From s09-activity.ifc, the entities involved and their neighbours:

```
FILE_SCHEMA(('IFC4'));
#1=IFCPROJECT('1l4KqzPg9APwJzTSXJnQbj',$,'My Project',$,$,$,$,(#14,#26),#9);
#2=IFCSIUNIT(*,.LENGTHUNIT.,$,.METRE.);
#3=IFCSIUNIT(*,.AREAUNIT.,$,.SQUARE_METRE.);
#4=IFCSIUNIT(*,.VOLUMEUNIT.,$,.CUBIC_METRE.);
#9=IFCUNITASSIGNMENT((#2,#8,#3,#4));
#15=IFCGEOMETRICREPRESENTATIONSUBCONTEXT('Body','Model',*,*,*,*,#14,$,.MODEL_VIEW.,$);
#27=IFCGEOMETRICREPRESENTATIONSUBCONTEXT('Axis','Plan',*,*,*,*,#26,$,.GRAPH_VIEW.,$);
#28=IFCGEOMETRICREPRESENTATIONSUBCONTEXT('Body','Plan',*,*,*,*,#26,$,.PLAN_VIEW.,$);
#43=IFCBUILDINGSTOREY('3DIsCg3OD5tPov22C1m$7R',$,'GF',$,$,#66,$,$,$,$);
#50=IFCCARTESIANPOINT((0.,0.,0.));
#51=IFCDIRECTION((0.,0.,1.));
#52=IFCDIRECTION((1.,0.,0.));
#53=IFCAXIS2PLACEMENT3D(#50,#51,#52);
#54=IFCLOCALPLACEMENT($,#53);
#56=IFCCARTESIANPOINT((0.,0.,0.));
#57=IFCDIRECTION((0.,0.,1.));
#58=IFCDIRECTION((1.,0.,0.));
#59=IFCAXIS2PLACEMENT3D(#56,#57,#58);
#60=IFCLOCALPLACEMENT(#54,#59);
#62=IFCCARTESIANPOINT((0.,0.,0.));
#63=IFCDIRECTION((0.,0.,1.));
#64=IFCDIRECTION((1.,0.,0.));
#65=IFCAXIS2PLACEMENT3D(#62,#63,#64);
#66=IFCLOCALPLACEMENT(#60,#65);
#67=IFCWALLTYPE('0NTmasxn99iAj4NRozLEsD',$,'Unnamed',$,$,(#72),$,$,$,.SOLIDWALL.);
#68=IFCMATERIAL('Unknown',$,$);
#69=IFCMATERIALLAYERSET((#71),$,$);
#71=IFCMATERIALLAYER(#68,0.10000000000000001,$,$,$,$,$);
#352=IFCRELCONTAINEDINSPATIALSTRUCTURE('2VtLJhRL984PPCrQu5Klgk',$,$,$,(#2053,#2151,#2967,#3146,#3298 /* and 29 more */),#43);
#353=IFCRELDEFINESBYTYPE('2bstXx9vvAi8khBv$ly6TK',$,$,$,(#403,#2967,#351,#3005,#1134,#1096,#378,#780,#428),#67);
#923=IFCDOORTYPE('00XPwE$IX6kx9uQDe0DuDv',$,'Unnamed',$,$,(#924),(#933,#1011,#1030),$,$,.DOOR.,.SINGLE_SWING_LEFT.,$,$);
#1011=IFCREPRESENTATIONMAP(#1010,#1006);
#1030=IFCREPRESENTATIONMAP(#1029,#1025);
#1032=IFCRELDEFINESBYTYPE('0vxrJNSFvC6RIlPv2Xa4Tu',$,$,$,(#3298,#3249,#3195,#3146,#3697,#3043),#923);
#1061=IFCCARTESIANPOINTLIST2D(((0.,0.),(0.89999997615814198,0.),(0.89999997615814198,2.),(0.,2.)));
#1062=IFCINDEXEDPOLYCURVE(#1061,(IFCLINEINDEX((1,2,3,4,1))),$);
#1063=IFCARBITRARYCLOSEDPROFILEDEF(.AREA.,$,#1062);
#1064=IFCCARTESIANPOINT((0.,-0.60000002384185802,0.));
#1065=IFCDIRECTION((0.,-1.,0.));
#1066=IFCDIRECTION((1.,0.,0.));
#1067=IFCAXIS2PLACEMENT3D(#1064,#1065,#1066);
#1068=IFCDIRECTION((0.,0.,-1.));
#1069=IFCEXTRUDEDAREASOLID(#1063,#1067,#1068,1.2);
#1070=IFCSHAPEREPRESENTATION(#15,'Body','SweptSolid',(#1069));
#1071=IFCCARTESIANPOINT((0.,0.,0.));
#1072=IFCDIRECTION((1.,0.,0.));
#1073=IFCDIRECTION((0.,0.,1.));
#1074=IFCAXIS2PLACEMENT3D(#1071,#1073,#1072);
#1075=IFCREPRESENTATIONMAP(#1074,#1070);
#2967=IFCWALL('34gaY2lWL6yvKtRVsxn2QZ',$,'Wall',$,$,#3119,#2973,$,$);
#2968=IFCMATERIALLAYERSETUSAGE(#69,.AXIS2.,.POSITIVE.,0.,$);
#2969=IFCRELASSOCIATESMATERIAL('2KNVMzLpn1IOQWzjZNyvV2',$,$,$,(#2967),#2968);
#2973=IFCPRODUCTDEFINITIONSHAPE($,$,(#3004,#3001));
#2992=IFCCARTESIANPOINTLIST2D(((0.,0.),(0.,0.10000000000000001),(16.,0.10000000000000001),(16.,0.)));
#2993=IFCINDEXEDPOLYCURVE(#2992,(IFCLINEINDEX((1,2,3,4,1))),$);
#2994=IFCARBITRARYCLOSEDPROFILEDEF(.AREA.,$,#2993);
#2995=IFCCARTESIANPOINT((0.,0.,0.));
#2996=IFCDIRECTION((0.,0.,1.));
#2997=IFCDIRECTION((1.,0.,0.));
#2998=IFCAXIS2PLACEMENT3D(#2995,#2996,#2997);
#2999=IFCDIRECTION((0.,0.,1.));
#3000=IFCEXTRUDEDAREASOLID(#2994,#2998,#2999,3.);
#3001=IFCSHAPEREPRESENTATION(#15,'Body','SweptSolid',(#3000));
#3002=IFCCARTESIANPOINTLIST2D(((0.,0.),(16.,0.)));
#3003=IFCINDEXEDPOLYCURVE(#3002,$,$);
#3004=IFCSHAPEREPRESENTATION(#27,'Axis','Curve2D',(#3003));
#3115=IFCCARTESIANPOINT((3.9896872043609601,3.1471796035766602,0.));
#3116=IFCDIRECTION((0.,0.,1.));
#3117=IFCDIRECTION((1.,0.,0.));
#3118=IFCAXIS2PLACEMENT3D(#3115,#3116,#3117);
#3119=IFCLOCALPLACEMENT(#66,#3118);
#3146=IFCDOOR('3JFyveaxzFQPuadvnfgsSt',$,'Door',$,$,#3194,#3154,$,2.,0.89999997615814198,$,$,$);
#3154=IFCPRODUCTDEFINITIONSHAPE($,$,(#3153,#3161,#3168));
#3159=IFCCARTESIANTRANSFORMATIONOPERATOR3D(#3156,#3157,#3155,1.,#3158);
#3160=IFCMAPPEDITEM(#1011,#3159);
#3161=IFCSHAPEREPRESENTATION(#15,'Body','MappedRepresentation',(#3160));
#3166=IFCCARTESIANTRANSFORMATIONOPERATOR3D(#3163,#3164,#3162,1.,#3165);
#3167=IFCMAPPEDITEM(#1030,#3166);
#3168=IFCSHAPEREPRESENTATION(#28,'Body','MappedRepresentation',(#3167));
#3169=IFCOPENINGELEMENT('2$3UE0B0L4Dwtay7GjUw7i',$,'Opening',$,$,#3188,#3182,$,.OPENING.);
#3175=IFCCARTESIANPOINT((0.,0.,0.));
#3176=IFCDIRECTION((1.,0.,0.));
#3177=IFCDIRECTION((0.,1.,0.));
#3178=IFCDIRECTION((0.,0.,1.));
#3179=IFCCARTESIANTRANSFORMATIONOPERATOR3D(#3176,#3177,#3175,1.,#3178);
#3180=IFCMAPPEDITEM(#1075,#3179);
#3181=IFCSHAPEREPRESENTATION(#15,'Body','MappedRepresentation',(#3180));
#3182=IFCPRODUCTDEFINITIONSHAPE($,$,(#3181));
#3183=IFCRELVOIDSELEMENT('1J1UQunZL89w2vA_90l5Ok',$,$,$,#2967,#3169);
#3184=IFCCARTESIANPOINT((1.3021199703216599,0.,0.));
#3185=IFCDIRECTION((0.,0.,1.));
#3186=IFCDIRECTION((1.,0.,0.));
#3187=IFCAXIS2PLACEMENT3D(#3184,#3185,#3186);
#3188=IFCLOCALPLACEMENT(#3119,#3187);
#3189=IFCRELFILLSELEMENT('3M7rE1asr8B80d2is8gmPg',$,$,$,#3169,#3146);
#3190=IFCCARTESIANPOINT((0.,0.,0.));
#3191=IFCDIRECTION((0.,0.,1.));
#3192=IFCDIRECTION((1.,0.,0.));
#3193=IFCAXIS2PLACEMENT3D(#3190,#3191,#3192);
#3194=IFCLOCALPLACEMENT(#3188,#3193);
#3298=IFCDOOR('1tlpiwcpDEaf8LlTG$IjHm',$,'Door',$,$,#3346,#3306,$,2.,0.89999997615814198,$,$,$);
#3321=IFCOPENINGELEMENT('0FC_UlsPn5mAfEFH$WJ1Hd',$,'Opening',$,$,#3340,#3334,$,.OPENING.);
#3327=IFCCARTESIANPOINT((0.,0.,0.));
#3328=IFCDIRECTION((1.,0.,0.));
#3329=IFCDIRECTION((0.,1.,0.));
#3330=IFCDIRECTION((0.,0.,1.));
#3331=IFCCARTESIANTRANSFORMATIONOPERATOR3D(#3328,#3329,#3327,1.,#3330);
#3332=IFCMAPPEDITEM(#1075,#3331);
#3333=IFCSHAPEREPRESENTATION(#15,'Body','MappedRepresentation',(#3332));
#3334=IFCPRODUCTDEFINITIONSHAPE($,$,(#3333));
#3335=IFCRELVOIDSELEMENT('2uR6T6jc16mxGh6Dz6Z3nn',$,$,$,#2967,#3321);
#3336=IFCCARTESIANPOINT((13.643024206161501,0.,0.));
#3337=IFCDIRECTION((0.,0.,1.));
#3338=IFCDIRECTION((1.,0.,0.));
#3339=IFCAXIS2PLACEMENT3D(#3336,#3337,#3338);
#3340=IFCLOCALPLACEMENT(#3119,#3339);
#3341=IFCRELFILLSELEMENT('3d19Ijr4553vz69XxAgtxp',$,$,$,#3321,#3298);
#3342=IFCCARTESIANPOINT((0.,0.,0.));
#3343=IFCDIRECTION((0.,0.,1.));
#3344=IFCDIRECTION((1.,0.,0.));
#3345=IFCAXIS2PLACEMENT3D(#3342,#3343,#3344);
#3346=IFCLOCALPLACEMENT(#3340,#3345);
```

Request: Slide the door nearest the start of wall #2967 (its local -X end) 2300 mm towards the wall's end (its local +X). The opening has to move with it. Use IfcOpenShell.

```python
import ifcopenshell
import ifcopenshell.api.geometry
import ifcopenshell.util.placement
import ifcopenshell.util.unit

model = ifcopenshell.open("s09-activity.ifc")
unit_scale = ifcopenshell.util.unit.calculate_unit_scale(model)

door = model.by_guid("3JFyveaxzFQPuadvnfgsSt")
opening = door.FillsVoids[0].RelatingOpeningElement
wall = opening.VoidsElements[0].RelatingBuildingElement

wall_matrix = ifcopenshell.util.placement.get_local_placement(wall.ObjectPlacement)
shift = wall_matrix[:3, 0] * 2.3 / unit_scale
before = ifcopenshell.util.placement.get_local_placement(door.ObjectPlacement)[:3, 3].copy()

# The door is placed relative to its opening, so it follows when the opening moves.
matrix = ifcopenshell.util.placement.get_local_placement(opening.ObjectPlacement)
matrix[:3, 3] += shift
ifcopenshell.api.geometry.edit_object_placement(
    model, product=opening, matrix=matrix, is_si=False, should_transform_children=True
)

after = ifcopenshell.util.placement.get_local_placement(door.ObjectPlacement)[:3, 3]
print("door moved by", (after - before).round(3) + 0.0)

model.write("s09-activity_rev.ifc")
```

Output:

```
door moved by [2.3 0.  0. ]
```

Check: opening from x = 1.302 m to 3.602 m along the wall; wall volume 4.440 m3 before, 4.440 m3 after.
